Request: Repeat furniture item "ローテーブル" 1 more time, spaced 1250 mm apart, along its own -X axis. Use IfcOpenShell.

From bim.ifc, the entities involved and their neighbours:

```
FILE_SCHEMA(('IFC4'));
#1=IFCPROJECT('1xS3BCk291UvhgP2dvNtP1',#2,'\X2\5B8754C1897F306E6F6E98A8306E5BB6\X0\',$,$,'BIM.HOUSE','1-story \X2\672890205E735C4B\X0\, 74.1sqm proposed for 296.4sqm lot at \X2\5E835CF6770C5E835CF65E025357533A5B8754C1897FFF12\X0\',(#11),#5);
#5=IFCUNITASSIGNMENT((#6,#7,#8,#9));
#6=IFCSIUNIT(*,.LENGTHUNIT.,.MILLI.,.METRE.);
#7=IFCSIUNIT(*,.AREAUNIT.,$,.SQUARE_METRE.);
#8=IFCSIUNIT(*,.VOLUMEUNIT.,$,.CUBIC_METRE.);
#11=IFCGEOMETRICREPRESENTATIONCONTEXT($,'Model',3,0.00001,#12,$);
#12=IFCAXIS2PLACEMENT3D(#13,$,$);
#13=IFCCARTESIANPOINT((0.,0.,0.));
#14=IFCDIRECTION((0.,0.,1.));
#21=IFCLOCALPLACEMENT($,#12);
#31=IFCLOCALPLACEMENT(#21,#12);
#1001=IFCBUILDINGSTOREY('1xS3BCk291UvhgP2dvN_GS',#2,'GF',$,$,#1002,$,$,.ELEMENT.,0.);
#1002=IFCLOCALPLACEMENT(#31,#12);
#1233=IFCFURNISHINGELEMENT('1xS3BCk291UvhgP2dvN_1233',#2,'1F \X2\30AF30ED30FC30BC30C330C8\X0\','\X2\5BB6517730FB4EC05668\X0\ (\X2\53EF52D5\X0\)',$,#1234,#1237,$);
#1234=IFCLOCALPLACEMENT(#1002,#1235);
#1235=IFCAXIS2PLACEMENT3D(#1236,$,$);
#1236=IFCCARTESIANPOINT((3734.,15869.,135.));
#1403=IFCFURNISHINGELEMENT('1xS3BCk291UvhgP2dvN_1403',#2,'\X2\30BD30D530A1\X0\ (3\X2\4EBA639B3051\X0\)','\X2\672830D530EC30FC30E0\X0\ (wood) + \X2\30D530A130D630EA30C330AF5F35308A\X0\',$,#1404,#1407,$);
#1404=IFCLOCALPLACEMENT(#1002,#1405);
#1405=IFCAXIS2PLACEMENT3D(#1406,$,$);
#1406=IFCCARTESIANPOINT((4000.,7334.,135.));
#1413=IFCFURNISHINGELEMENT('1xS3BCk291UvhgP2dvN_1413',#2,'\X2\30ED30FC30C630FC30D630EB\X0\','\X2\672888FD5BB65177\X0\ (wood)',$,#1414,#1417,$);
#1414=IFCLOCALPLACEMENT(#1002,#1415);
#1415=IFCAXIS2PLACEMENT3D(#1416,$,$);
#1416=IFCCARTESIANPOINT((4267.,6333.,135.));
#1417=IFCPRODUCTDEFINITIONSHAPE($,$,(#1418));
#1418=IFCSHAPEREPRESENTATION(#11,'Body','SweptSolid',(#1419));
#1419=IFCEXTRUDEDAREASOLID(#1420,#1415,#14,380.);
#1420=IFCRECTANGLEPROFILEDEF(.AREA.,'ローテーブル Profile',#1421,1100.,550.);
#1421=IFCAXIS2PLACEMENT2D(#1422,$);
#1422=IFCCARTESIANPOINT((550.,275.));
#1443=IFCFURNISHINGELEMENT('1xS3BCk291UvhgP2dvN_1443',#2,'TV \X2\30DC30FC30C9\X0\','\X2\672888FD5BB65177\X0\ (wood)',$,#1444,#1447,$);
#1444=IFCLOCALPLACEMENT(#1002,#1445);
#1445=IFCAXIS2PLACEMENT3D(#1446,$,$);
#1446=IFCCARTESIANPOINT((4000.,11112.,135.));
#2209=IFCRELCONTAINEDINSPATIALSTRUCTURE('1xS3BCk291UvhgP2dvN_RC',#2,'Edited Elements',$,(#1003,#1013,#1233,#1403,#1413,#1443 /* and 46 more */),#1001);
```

```python
import ifcopenshell
import ifcopenshell.api.geometry
import ifcopenshell.api.root
import ifcopenshell.util.element
import ifcopenshell.util.placement

model = ifcopenshell.open("bim.ifc")


def reuse_history(source, copy):
    """copy_class also copies each property set's owner history, people and application; keep the originals."""
    for rel in copy.IsDefinedBy:
        if rel.is_a("IfcRelDefinesByProperties") and (history := rel.RelatingPropertyDefinition.OwnerHistory):
            rel.RelatingPropertyDefinition.OwnerHistory = source.OwnerHistory
            ifcopenshell.util.element.remove_deep2(model, history)


source = model.by_id(1413)
base = ifcopenshell.util.placement.get_local_placement(source.ObjectPlacement)
step = -base[:3, 0] * 1250.0

for i in range(1, 2):
    copy = ifcopenshell.api.root.copy_class(model, product=source)
    copy.Representation = ifcopenshell.util.element.copy_deep(
        model, source.Representation, exclude=["IfcGeometricRepresentationContext", "IfcRepresentationMap"]
    )
    reuse_history(source, copy)
    matrix = base.copy()
    matrix[:3, 3] += i * step
    print("added at", matrix[:3, 3].round(3) + 0.0)
    ifcopenshell.api.geometry.edit_object_placement(model, product=copy, matrix=matrix, is_si=False)

model.write("bim_v2.ifc")
```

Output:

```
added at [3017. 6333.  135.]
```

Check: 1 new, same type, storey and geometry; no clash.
